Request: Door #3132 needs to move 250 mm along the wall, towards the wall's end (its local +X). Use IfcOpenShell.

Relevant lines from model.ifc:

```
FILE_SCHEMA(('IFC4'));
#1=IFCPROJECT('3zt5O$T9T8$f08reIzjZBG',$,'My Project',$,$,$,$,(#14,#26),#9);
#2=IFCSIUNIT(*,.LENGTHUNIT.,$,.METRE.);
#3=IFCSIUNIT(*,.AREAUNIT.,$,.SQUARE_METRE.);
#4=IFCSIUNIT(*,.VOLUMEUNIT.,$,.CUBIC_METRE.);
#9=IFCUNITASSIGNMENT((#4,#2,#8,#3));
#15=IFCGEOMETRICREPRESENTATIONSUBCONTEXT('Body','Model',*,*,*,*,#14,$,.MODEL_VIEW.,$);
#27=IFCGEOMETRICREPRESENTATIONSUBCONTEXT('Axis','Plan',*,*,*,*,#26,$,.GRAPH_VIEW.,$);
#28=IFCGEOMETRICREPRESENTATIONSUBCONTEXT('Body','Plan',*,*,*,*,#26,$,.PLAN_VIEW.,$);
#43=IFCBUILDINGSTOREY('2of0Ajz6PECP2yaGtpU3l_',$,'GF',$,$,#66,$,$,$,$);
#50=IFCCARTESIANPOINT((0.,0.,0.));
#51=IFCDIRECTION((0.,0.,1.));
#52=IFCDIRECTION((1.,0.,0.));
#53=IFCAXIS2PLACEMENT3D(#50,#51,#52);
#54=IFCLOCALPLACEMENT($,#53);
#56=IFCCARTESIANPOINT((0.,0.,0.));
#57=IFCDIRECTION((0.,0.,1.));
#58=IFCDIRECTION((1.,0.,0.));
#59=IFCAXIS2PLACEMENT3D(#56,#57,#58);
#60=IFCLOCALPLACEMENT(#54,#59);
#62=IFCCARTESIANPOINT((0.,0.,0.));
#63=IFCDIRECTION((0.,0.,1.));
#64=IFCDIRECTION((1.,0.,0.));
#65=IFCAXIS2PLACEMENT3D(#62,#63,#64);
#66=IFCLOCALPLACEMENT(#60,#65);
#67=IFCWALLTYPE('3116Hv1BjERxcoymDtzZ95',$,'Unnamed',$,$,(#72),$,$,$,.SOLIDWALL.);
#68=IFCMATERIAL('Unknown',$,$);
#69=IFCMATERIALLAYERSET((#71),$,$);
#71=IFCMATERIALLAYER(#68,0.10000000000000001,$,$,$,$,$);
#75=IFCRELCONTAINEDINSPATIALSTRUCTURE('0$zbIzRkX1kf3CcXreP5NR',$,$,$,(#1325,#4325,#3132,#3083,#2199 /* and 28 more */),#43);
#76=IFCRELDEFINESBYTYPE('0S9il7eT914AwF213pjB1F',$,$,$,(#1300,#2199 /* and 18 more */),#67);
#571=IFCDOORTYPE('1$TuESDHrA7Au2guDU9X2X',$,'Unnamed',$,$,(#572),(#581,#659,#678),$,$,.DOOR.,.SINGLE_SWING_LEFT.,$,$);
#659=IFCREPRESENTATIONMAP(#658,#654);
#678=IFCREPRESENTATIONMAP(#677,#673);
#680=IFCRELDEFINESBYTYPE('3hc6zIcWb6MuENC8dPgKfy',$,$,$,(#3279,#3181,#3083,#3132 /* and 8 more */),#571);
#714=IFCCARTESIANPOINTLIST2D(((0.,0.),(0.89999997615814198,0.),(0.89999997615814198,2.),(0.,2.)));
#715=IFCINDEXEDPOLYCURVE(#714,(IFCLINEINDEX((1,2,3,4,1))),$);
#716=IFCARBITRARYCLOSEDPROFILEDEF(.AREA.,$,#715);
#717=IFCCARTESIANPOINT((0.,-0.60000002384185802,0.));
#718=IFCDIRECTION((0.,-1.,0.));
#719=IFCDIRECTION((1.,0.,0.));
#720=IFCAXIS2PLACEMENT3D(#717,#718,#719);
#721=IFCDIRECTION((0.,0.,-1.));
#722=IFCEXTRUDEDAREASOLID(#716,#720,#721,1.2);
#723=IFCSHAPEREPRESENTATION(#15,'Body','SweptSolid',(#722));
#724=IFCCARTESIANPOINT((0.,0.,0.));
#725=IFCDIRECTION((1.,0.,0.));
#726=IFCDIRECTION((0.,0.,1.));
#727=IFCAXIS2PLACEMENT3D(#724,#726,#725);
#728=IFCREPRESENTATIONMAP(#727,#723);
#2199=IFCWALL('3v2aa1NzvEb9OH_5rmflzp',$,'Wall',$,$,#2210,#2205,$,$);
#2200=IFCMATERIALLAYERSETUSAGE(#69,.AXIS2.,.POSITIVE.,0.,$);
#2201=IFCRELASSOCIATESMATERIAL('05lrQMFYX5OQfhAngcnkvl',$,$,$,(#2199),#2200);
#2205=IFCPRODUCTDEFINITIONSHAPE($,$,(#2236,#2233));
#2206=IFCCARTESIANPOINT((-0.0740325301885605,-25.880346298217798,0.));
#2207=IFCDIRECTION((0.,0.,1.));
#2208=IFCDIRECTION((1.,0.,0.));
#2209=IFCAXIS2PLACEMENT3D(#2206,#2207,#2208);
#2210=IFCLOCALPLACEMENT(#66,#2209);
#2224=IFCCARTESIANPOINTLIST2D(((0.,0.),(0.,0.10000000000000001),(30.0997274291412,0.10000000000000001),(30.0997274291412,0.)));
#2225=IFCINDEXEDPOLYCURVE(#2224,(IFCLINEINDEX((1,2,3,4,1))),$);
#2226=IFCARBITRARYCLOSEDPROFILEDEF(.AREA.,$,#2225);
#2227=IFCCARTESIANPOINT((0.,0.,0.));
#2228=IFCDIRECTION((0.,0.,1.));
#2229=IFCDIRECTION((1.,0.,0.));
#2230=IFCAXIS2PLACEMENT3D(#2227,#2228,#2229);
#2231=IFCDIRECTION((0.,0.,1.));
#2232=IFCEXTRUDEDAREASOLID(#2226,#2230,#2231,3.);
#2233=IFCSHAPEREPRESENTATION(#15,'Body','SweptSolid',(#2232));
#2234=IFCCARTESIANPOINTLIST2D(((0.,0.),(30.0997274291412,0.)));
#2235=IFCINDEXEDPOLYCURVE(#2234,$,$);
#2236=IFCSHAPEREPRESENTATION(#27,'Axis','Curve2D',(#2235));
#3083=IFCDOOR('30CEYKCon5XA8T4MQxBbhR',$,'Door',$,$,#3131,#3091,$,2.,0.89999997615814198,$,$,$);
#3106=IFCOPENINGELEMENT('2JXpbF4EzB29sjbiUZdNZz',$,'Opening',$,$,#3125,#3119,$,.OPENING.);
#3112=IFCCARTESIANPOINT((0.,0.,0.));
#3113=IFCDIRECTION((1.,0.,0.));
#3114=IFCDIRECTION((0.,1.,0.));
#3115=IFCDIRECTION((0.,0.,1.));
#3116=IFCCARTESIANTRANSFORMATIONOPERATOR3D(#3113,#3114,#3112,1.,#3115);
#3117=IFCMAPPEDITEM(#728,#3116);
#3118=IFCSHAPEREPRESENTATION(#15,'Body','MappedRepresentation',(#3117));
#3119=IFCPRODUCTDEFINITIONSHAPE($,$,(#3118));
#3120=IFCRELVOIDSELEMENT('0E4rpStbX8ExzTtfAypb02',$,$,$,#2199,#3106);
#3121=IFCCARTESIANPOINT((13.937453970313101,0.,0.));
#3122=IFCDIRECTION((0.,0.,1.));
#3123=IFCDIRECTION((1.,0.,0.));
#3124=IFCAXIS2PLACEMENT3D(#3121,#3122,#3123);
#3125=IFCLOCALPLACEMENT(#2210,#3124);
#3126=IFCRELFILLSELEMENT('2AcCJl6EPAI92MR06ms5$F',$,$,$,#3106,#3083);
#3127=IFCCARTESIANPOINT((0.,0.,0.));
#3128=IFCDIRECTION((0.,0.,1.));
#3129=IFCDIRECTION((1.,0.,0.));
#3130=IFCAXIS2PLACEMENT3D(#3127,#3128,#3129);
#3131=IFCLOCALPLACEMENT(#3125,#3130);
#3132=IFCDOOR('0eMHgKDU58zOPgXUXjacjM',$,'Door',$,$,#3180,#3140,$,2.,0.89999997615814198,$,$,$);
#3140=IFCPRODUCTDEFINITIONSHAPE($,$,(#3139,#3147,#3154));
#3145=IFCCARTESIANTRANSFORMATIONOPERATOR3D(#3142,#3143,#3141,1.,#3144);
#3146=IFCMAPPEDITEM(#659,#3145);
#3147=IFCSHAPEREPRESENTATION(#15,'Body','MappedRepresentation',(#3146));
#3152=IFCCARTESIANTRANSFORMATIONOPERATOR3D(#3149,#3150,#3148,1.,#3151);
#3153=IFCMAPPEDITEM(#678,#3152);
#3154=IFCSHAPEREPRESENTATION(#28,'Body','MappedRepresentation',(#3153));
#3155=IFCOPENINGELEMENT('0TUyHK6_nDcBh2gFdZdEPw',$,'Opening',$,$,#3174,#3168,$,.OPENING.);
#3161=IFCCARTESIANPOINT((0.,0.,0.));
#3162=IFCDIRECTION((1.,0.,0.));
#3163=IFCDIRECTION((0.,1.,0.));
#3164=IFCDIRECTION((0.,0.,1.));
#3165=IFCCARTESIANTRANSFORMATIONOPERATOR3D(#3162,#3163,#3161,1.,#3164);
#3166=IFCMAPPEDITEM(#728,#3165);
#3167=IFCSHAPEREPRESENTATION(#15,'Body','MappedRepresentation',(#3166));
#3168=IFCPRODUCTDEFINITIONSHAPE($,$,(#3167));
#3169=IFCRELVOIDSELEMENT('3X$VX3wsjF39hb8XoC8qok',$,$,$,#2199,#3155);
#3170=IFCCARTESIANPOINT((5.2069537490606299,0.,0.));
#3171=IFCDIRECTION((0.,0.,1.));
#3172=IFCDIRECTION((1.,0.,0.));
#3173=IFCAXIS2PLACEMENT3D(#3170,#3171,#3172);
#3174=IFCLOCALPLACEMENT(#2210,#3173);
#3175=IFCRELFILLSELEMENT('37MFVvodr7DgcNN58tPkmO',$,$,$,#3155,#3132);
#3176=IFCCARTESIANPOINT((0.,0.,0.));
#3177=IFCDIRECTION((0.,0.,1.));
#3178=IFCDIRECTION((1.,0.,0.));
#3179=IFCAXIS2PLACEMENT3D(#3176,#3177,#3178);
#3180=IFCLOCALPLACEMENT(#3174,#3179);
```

```python
import ifcopenshell
import ifcopenshell.api.geometry
import ifcopenshell.util.placement

model = ifcopenshell.open("model.ifc")

door = model.by_guid("0eMHgKDU58zOPgXUXjacjM")
opening = door.FillsVoids[0].RelatingOpeningElement
wall = opening.VoidsElements[0].RelatingBuildingElement

wall_matrix = ifcopenshell.util.placement.get_local_placement(wall.ObjectPlacement)
shift = wall_matrix[:3, 0] * 0.25
before = ifcopenshell.util.placement.get_local_placement(door.ObjectPlacement)[:3, 3].copy()

# The door is placed relative to its opening, so it follows when the opening moves.
matrix = ifcopenshell.util.placement.get_local_placement(opening.ObjectPlacement)
matrix[:3, 3] += shift
ifcopenshell.api.geometry.edit_object_placement(
    model, product=opening, matrix=matrix, is_si=False, should_transform_children=True
)

after = ifcopenshell.util.placement.get_local_placement(door.ObjectPlacement)[:3, 3]
print("door moved by", (after - before).round(3) + 0.0)

model.write("model_edited.ifc")
```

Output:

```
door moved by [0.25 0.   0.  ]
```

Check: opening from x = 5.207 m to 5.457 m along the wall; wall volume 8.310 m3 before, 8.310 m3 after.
